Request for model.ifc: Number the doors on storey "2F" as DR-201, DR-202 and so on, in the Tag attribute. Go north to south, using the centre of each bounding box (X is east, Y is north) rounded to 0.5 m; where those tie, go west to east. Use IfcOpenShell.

First a look at what the model holds.

```python
import ifcopenshell
import ifcopenshell.util.element
import ifcopenshell.util.placement

model = ifcopenshell.open("model.ifc")
print(model.schema)
storey = next(s for s in model.by_type("IfcBuildingStorey") if s.Name == "2F")
doors = [e for e in ifcopenshell.util.element.get_decomposition(storey) if e.is_a("IfcDoor")]
for e in sorted(doors, key=lambda e: e.id()):
    origin = ifcopenshell.util.placement.get_local_placement(e.ObjectPlacement)[:3, 3]
    print(e.id(), e.Tag, e.Name, origin.round(2) + 0.0, sep=" | ")
```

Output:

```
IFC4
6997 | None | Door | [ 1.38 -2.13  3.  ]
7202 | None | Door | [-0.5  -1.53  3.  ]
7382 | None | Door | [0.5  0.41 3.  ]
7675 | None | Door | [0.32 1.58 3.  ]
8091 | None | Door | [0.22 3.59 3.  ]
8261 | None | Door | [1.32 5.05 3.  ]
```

```python
import ifcopenshell
import ifcopenshell.geom
import ifcopenshell.util.element
import ifcopenshell.util.shape

model = ifcopenshell.open("model.ifc")
settings = ifcopenshell.geom.settings()
settings.set("use-world-coords", True)


def centre(element):
    shape = ifcopenshell.geom.create_shape(settings, element)
    return ifcopenshell.util.shape.get_bbox_centroid(shape.geometry)


storey = next(s for s in model.by_type("IfcBuildingStorey") if s.Name == "2F")
doors = [e for e in ifcopenshell.util.element.get_decomposition(storey) if e.is_a("IfcDoor")]

# Insertion points can sit at a corner or the storey origin, so sort by the geometry (in metres).
centres = {e: centre(e) for e in doors}
doors.sort(key=lambda e: (-round(centres[e][1] / 0.5), centres[e][0]))

for i, e in enumerate(doors, start=1):
    number = f"DR-2{i:02d}"
    e.Tag = number
    print(e.id(), number)

model.write("model_edited.ifc")
```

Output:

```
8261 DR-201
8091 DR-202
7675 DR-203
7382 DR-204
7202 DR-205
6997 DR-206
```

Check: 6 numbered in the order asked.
